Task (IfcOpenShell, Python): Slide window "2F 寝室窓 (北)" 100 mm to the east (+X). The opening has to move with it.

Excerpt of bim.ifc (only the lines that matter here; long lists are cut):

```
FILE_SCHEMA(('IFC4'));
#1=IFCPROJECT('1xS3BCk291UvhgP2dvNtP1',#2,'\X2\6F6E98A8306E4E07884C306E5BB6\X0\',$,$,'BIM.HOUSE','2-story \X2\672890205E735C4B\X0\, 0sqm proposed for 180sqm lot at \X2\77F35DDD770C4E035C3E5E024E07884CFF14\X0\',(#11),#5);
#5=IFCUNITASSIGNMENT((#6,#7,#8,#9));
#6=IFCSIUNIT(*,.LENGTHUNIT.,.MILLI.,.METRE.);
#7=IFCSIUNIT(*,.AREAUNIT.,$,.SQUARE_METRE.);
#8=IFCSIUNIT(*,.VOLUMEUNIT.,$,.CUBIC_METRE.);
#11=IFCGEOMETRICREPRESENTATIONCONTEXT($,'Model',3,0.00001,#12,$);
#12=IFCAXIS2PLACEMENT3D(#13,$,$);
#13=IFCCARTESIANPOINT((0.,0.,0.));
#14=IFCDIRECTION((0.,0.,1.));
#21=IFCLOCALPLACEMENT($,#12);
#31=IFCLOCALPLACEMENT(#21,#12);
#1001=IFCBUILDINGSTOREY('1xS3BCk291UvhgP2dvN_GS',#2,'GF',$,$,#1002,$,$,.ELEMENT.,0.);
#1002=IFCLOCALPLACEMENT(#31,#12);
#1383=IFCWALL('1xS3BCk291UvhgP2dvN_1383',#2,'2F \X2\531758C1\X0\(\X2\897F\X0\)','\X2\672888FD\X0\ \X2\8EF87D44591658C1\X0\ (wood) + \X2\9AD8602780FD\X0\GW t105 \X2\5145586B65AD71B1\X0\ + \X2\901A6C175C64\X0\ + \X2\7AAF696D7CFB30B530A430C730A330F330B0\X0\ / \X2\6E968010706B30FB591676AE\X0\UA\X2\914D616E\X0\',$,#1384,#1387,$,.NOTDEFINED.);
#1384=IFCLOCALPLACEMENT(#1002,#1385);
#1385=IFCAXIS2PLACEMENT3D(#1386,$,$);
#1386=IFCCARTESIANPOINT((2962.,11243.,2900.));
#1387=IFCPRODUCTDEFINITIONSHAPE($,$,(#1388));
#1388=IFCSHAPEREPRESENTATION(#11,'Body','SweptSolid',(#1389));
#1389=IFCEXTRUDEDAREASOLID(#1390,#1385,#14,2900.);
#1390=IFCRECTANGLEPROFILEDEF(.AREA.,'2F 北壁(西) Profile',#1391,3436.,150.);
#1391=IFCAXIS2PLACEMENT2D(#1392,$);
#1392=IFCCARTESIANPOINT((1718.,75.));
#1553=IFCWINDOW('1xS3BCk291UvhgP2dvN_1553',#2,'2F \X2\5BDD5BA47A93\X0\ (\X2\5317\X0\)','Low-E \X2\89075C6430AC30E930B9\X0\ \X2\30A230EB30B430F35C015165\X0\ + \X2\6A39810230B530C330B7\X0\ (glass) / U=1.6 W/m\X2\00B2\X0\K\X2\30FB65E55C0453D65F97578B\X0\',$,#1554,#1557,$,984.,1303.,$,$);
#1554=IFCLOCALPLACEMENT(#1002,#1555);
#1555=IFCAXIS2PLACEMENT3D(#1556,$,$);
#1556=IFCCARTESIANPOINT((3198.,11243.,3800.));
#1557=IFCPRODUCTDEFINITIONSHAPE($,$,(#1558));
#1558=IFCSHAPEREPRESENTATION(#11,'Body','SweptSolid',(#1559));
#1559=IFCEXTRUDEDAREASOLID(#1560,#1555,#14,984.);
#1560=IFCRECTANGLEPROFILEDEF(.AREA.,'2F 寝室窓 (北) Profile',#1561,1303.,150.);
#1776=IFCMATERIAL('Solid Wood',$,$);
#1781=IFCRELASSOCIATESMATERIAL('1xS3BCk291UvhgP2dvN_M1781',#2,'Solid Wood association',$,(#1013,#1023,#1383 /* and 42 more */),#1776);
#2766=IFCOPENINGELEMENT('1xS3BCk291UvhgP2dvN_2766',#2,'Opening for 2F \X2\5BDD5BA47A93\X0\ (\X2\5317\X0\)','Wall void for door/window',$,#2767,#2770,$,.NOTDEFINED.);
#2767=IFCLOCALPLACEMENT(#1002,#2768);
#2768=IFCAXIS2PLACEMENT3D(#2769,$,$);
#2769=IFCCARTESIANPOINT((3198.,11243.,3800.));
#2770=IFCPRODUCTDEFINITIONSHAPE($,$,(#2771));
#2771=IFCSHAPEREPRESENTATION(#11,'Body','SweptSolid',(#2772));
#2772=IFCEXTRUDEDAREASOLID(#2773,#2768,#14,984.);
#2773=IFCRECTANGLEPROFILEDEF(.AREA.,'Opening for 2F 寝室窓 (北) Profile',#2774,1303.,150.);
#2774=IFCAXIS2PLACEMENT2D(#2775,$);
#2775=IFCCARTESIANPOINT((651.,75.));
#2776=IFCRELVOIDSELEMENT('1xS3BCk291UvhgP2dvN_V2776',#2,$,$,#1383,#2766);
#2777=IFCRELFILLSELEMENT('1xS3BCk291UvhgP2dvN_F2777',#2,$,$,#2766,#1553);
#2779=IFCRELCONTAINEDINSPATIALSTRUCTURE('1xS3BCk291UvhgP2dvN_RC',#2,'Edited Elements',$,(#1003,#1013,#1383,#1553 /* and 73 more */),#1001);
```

```python
import ifcopenshell
import ifcopenshell.api.geometry
import ifcopenshell.util.placement
import ifcopenshell.util.unit

model = ifcopenshell.open("bim.ifc")
unit_scale = ifcopenshell.util.unit.calculate_unit_scale(model)

window = model.by_guid("1xS3BCk291UvhgP2dvN_1553")
opening = window.FillsVoids[0].RelatingOpeningElement
wall = opening.VoidsElements[0].RelatingBuildingElement

wall_matrix = ifcopenshell.util.placement.get_local_placement(wall.ObjectPlacement)
shift = wall_matrix[:3, 0] * 0.1 / unit_scale
before = ifcopenshell.util.placement.get_local_placement(window.ObjectPlacement)[:3, 3].copy()

# The window is not placed relative to its opening, so move both.
for product in (opening, window):
    matrix = ifcopenshell.util.placement.get_local_placement(product.ObjectPlacement)
    matrix[:3, 3] += shift
    ifcopenshell.api.geometry.edit_object_placement(model, product=product, matrix=matrix, is_si=False)

after = ifcopenshell.util.placement.get_local_placement(window.ObjectPlacement)[:3, 3]
print("window moved by", (after - before).round(3) + 0.0)

model.write("bim_updated.ifc")
```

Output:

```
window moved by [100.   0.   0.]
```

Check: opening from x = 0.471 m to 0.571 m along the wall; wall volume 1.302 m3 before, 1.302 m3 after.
